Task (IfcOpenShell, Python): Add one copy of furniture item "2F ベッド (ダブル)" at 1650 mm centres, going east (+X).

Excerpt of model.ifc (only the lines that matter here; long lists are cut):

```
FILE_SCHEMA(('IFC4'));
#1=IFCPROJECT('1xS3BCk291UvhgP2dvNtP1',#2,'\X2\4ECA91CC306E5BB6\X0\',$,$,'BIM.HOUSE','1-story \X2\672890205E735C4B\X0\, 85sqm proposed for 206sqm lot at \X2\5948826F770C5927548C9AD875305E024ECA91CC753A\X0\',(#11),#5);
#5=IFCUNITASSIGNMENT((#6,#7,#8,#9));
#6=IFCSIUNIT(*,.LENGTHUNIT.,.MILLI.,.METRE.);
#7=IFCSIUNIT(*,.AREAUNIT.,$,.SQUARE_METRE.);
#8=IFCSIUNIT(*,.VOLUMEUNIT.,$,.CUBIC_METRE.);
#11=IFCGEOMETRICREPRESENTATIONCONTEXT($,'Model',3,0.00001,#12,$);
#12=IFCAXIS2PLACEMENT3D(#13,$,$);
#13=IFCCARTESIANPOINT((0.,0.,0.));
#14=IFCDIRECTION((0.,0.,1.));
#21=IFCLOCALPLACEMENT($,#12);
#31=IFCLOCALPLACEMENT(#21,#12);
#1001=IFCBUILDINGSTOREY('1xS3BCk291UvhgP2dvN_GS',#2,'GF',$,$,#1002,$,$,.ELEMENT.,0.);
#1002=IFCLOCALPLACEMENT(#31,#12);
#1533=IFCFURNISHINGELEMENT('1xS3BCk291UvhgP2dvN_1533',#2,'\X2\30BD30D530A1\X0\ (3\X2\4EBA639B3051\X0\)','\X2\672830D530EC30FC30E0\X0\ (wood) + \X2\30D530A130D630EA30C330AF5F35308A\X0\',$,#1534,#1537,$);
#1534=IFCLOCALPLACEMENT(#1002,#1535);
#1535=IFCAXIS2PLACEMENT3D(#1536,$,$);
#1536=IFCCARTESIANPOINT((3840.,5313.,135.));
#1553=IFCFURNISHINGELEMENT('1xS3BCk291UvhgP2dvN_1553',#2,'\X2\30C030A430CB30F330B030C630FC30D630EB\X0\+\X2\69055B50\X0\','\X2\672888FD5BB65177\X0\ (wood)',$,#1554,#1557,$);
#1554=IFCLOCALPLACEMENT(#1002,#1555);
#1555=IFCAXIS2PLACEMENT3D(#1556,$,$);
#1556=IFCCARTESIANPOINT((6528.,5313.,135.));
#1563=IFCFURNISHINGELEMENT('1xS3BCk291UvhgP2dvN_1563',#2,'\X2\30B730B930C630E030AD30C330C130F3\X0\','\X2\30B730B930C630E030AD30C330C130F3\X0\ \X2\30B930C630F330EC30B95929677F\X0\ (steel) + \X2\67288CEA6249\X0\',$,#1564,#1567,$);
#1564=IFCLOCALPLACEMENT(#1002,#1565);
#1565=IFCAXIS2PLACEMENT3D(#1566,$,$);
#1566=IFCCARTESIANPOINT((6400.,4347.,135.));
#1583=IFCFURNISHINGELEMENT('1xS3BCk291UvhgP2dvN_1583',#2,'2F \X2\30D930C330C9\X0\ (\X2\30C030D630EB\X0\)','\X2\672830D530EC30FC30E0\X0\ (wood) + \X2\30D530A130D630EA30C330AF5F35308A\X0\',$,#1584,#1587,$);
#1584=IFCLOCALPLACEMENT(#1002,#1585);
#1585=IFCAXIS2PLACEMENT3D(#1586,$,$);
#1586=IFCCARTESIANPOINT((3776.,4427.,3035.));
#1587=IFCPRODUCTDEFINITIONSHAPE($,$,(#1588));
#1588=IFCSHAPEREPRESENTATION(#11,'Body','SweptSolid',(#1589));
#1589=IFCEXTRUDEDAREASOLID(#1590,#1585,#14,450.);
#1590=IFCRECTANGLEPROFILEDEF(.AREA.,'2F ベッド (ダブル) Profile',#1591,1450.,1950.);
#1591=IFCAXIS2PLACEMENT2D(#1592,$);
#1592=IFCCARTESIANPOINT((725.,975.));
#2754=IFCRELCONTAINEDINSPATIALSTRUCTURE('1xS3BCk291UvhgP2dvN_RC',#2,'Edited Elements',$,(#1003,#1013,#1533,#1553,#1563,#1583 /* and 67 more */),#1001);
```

```python
import numpy as np
import ifcopenshell
import ifcopenshell.api.geometry
import ifcopenshell.api.root
import ifcopenshell.util.element
import ifcopenshell.util.placement

model = ifcopenshell.open("model.ifc")


def reuse_history(source, copy):
    """copy_class also copies each property set's owner history, people and application; keep the originals."""
    for rel in copy.IsDefinedBy:
        if rel.is_a("IfcRelDefinesByProperties") and (history := rel.RelatingPropertyDefinition.OwnerHistory):
            rel.RelatingPropertyDefinition.OwnerHistory = source.OwnerHistory
            ifcopenshell.util.element.remove_deep2(model, history)


source = model.by_guid("1xS3BCk291UvhgP2dvN_1583")
base = ifcopenshell.util.placement.get_local_placement(source.ObjectPlacement)
step = np.array([1.0, 0.0, 0.0]) * 1650.0

for i in range(1, 2):
    copy = ifcopenshell.api.root.copy_class(model, product=source)
    copy.Representation = ifcopenshell.util.element.copy_deep(
        model, source.Representation, exclude=["IfcGeometricRepresentationContext", "IfcRepresentationMap"]
    )
    reuse_history(source, copy)
    matrix = base.copy()
    matrix[:3, 3] += i * step
    print("added at", matrix[:3, 3].round(3) + 0.0)
    ifcopenshell.api.geometry.edit_object_placement(model, product=copy, matrix=matrix, is_si=False)

model.write("model_updated.ifc")
```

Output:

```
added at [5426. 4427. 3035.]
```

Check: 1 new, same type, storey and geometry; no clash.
